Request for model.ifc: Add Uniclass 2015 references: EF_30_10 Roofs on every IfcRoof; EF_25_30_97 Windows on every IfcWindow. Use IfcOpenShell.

First a look at what the model holds.

```python
import ifcopenshell

model = ifcopenshell.open("model.ifc")
print(model.schema)
print("classifications:", [c.Name for c in model.by_type("IfcClassification")])
for ifc_class in ("IfcDoor", "IfcRoof", "IfcStair", "IfcWall", "IfcWindow"):
    print(ifc_class, len(model.by_type(ifc_class)))
```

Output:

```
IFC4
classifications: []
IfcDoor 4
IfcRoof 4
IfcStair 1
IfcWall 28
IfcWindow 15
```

```python
import ifcopenshell
import ifcopenshell.api.classification

model = ifcopenshell.open("model.ifc")

system = ifcopenshell.api.classification.add_classification(model, classification="Uniclass 2015")

codes = {
    "IfcRoof": ("EF_30_10", "Roofs"),
    "IfcWindow": ("EF_25_30_97", "Windows"),
}
for ifc_class, (code, name) in codes.items():
    products = model.by_type(ifc_class)
    ifcopenshell.api.classification.add_reference(
        model, products=products, classification=system, identification=code, name=name
    )
    print(code, len(products))

model.write("model_rev.ifc")
```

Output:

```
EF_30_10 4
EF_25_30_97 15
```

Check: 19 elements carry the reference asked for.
